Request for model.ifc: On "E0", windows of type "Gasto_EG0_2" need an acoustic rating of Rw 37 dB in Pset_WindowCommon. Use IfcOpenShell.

First a look at what the model holds.

```python
import ifcopenshell
import ifcopenshell.util.element

model = ifcopenshell.open("model.ifc")
print(model.schema)
storey = next(s for s in model.by_type("IfcBuildingStorey") if s.Name == "E0")
windows = [e for e in ifcopenshell.util.element.get_decomposition(storey) if e.is_a("IfcWindow")]
seen = {}
for e in windows:
    element_type = ifcopenshell.util.element.get_type(e)
    key = (element_type.Name if element_type != e and element_type else None, ifcopenshell.util.element.get_pset(e, "Pset_WindowCommon", "AcousticRating"))
    seen[key] = seen.get(key, 0) + 1
for (name, value), count in sorted(seen.items(), key=str):
    print(count, "x", name, "|", value)
```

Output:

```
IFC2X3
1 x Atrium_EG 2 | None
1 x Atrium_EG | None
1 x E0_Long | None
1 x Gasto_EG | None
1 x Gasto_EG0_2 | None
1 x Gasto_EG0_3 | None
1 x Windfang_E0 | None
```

```python
import ifcopenshell
import ifcopenshell.api.pset
import ifcopenshell.util.element

model = ifcopenshell.open("model.ifc")

storey = next(s for s in model.by_type("IfcBuildingStorey") if s.Name == "E0")
windows = [e for e in ifcopenshell.util.element.get_decomposition(storey) if e.is_a("IfcWindow")]

count = 0
for e in windows:
    element_type = ifcopenshell.util.element.get_type(e)
    if element_type in (None, e) or element_type.Name != "Gasto_EG0_2":
        continue
    # add_pset returns the element's existing set when there is one.
    pset = ifcopenshell.api.pset.add_pset(model, product=e, name="Pset_WindowCommon")
    ifcopenshell.api.pset.edit_pset(model, pset=pset, properties={"AcousticRating": "Rw 37 dB"})
    count += 1

print(count, "windows updated")

model.write("model_v2.ifc")
```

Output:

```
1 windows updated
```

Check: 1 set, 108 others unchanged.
